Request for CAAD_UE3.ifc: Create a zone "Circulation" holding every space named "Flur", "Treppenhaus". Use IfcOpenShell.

First a look at what the model holds.

```python
import ifcopenshell

model = ifcopenshell.open("CAAD_UE3.ifc")
print(model.schema)
seen = {}
for space in model.by_type("IfcSpace"):
    seen[space.LongName] = seen.get(space.LongName, 0) + 1
for name, count in sorted(seen.items(), key=str):
    print(count, "x", name)
print("zones:", [z.Name for z in model.by_type("IfcZone")][:20])
```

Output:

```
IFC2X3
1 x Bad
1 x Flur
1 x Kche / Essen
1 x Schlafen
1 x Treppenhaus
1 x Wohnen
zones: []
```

```python
import ifcopenshell
import ifcopenshell.api.group
import ifcopenshell.api.root

model = ifcopenshell.open("CAAD_UE3.ifc")

names = {"Flur", "Treppenhaus"}
spaces = [s for s in model.by_type("IfcSpace") if s.LongName in names]

zone = ifcopenshell.api.root.create_entity(model, ifc_class="IfcZone", name="Circulation")
ifcopenshell.api.group.assign_group(model, products=spaces, group=zone)
print(len(spaces), "spaces in", zone.Name)

model.write("CAAD_UE3_rev.ifc")
```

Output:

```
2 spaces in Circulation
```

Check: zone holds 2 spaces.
